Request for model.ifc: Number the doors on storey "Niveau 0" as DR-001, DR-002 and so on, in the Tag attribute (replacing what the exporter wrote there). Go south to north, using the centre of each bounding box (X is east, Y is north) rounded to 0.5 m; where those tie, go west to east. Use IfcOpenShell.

First a look at what the model holds.

```python
import ifcopenshell
import ifcopenshell.util.element
import ifcopenshell.util.placement

model = ifcopenshell.open("model.ifc")
print(model.schema)
storey = next(s for s in model.by_type("IfcBuildingStorey") if s.Name == "Niveau 0")
doors = [e for e in ifcopenshell.util.element.get_decomposition(storey) if e.is_a("IfcDoor")]
for e in sorted(doors, key=lambda e: e.id()):
    origin = ifcopenshell.util.placement.get_local_placement(e.ObjectPlacement)[:3, 3]
    print(e.id(), e.Tag, e.Name, origin.round(2) + 0.0, sep=" | ")
```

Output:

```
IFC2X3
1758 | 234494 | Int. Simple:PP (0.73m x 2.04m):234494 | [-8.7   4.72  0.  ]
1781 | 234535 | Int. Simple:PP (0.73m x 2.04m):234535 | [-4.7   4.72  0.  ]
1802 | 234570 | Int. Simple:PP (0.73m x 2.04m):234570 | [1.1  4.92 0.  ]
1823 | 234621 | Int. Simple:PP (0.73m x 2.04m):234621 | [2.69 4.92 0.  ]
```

```python
import ifcopenshell
import ifcopenshell.geom
import ifcopenshell.util.element
import ifcopenshell.util.shape

model = ifcopenshell.open("model.ifc")
settings = ifcopenshell.geom.settings()
settings.set("use-world-coords", True)


def centre(element):
    shape = ifcopenshell.geom.create_shape(settings, element)
    return ifcopenshell.util.shape.get_bbox_centroid(shape.geometry)


storey = next(s for s in model.by_type("IfcBuildingStorey") if s.Name == "Niveau 0")
doors = [e for e in ifcopenshell.util.element.get_decomposition(storey) if e.is_a("IfcDoor")]

# Insertion points can sit at a corner or the storey origin, so sort by the geometry (in metres).
centres = {e: centre(e) for e in doors}
doors.sort(key=lambda e: (round(centres[e][1] / 0.5), centres[e][0]))

for i, e in enumerate(doors, start=1):
    number = f"DR-0{i:02d}"
    e.Tag = number
    print(e.id(), number)

model.write("model_rev.ifc")
```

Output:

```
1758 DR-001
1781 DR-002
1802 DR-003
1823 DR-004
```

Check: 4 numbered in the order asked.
